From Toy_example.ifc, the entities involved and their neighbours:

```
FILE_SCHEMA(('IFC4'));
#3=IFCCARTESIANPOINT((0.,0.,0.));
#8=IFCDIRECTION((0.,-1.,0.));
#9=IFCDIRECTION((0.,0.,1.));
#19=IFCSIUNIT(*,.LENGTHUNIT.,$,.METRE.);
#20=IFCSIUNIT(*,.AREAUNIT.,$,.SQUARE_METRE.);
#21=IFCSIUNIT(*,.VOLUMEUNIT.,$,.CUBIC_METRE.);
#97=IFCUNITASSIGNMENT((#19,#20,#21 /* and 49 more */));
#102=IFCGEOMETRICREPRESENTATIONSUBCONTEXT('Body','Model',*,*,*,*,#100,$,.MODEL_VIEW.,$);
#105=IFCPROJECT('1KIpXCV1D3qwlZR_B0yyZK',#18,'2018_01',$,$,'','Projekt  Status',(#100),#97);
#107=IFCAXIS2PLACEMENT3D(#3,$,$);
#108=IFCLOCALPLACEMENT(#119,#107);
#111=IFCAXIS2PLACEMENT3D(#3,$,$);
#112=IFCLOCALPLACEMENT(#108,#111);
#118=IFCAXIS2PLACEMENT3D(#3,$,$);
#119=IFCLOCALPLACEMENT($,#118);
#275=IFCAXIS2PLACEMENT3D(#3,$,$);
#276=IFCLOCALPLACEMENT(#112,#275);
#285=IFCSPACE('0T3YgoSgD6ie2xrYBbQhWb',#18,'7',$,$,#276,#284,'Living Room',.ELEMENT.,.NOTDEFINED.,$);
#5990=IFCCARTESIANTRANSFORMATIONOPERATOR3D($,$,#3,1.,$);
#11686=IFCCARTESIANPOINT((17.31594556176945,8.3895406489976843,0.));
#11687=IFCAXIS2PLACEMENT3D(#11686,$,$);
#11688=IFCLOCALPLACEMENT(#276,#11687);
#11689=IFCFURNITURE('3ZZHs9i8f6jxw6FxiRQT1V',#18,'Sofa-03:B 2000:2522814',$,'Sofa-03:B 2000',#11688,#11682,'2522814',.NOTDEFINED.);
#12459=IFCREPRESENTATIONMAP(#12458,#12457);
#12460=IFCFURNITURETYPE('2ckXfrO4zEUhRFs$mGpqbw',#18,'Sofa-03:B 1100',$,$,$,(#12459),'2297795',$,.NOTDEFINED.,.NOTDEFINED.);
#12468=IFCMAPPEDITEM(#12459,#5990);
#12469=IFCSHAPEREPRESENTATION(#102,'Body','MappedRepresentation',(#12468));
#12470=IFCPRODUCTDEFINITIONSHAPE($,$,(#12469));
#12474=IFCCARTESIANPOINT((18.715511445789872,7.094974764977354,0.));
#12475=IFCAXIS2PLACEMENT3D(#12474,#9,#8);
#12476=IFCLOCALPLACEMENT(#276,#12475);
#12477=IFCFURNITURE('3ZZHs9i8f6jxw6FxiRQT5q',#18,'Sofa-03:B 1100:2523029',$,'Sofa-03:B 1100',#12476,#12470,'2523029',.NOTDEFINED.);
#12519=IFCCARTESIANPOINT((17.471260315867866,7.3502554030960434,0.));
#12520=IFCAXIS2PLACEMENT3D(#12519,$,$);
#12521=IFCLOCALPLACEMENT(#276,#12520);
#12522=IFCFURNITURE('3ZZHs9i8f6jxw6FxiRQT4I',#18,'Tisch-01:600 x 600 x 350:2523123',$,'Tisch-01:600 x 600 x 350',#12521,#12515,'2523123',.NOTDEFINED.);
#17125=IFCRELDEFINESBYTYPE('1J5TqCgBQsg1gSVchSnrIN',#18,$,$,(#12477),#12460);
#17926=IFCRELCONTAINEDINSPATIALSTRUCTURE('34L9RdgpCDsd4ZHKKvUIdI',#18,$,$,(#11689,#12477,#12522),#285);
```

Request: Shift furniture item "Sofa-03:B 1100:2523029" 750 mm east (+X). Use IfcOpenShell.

```python
import ifcopenshell
import ifcopenshell.api.geometry
import ifcopenshell.util.placement

model = ifcopenshell.open("Toy_example.ifc")

item = model.by_id(12477)
matrix = ifcopenshell.util.placement.get_local_placement(item.ObjectPlacement)
matrix[0, 3] += 0.75
ifcopenshell.api.geometry.edit_object_placement(model, product=item, matrix=matrix, is_si=False)

print(ifcopenshell.util.placement.get_local_placement(item.ObjectPlacement).round(3) + 0.0)

model.write("Toy_example_edited.ifc")
```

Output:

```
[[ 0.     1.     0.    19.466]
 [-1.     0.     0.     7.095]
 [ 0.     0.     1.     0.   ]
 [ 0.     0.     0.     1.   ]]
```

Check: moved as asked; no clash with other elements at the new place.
